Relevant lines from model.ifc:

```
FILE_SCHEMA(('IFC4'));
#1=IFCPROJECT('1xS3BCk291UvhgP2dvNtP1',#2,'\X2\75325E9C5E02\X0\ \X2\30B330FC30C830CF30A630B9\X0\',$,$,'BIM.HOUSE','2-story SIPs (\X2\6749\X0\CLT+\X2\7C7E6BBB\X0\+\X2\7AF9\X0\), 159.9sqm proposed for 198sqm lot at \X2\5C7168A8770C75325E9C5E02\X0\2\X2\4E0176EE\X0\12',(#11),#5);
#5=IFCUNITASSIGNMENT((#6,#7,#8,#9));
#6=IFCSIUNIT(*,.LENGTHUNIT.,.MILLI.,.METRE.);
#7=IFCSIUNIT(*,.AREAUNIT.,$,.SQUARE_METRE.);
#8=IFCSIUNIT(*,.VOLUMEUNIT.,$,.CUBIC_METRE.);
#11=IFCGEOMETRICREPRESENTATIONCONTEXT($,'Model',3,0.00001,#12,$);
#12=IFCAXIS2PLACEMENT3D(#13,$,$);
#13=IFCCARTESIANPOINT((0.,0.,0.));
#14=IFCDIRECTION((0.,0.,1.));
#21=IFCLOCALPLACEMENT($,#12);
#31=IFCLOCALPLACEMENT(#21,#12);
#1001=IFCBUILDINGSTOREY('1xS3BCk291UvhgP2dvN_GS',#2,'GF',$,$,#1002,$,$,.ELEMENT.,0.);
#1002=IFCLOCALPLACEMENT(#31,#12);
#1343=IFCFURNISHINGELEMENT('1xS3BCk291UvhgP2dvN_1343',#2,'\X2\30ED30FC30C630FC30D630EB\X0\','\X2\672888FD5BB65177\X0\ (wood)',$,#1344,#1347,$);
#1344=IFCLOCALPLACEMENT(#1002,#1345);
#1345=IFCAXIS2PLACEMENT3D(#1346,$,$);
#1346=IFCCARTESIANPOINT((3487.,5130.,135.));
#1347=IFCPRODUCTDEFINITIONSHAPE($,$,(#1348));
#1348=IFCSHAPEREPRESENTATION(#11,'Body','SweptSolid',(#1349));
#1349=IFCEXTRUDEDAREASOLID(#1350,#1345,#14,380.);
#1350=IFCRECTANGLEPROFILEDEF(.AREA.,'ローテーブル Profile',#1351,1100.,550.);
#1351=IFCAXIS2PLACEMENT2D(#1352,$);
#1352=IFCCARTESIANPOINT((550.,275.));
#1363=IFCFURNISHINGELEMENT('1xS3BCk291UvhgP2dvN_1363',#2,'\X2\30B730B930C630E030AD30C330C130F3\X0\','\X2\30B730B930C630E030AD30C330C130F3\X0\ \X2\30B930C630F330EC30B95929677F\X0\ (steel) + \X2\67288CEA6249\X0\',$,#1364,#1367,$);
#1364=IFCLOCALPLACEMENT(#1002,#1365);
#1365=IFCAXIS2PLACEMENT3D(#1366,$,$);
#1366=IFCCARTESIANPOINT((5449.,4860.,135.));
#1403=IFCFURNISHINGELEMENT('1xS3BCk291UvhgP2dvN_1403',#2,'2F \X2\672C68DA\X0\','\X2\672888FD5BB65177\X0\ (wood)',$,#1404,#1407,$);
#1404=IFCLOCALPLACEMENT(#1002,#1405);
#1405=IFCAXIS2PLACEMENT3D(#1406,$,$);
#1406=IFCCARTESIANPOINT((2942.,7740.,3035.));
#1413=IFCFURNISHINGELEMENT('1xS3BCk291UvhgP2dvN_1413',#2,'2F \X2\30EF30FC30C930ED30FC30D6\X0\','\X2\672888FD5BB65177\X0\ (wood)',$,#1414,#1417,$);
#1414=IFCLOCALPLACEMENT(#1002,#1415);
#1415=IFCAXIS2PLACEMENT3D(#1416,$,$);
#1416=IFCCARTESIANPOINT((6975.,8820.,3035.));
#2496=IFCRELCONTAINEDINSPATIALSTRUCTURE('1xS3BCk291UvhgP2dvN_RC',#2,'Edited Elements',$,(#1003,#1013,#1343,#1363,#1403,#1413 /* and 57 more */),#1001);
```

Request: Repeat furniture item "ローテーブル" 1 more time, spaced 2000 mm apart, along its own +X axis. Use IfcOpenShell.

```python
import ifcopenshell
import ifcopenshell.api.geometry
import ifcopenshell.api.root
import ifcopenshell.util.element
import ifcopenshell.util.placement
import ifcopenshell.util.unit

model = ifcopenshell.open("model.ifc")
unit_scale = ifcopenshell.util.unit.calculate_unit_scale(model)


def reuse_history(source, copy):
    """copy_class also copies each property set's owner history, people and application; keep the originals."""
    for rel in copy.IsDefinedBy:
        if rel.is_a("IfcRelDefinesByProperties") and (history := rel.RelatingPropertyDefinition.OwnerHistory):
            rel.RelatingPropertyDefinition.OwnerHistory = source.OwnerHistory
            ifcopenshell.util.element.remove_deep2(model, history)


source = model.by_guid("1xS3BCk291UvhgP2dvN_1343")
base = ifcopenshell.util.placement.get_local_placement(source.ObjectPlacement)
step = base[:3, 0] * 2 / unit_scale

for i in range(1, 2):
    copy = ifcopenshell.api.root.copy_class(model, product=source)
    copy.Representation = ifcopenshell.util.element.copy_deep(
        model, source.Representation, exclude=["IfcGeometricRepresentationContext", "IfcRepresentationMap"]
    )
    reuse_history(source, copy)
    matrix = base.copy()
    matrix[:3, 3] += i * step
    print("added at", matrix[:3, 3].round(3) + 0.0)
    ifcopenshell.api.geometry.edit_object_placement(model, product=copy, matrix=matrix, is_si=False)

model.write("model_edited.ifc")
```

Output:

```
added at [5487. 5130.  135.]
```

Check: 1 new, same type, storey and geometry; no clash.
